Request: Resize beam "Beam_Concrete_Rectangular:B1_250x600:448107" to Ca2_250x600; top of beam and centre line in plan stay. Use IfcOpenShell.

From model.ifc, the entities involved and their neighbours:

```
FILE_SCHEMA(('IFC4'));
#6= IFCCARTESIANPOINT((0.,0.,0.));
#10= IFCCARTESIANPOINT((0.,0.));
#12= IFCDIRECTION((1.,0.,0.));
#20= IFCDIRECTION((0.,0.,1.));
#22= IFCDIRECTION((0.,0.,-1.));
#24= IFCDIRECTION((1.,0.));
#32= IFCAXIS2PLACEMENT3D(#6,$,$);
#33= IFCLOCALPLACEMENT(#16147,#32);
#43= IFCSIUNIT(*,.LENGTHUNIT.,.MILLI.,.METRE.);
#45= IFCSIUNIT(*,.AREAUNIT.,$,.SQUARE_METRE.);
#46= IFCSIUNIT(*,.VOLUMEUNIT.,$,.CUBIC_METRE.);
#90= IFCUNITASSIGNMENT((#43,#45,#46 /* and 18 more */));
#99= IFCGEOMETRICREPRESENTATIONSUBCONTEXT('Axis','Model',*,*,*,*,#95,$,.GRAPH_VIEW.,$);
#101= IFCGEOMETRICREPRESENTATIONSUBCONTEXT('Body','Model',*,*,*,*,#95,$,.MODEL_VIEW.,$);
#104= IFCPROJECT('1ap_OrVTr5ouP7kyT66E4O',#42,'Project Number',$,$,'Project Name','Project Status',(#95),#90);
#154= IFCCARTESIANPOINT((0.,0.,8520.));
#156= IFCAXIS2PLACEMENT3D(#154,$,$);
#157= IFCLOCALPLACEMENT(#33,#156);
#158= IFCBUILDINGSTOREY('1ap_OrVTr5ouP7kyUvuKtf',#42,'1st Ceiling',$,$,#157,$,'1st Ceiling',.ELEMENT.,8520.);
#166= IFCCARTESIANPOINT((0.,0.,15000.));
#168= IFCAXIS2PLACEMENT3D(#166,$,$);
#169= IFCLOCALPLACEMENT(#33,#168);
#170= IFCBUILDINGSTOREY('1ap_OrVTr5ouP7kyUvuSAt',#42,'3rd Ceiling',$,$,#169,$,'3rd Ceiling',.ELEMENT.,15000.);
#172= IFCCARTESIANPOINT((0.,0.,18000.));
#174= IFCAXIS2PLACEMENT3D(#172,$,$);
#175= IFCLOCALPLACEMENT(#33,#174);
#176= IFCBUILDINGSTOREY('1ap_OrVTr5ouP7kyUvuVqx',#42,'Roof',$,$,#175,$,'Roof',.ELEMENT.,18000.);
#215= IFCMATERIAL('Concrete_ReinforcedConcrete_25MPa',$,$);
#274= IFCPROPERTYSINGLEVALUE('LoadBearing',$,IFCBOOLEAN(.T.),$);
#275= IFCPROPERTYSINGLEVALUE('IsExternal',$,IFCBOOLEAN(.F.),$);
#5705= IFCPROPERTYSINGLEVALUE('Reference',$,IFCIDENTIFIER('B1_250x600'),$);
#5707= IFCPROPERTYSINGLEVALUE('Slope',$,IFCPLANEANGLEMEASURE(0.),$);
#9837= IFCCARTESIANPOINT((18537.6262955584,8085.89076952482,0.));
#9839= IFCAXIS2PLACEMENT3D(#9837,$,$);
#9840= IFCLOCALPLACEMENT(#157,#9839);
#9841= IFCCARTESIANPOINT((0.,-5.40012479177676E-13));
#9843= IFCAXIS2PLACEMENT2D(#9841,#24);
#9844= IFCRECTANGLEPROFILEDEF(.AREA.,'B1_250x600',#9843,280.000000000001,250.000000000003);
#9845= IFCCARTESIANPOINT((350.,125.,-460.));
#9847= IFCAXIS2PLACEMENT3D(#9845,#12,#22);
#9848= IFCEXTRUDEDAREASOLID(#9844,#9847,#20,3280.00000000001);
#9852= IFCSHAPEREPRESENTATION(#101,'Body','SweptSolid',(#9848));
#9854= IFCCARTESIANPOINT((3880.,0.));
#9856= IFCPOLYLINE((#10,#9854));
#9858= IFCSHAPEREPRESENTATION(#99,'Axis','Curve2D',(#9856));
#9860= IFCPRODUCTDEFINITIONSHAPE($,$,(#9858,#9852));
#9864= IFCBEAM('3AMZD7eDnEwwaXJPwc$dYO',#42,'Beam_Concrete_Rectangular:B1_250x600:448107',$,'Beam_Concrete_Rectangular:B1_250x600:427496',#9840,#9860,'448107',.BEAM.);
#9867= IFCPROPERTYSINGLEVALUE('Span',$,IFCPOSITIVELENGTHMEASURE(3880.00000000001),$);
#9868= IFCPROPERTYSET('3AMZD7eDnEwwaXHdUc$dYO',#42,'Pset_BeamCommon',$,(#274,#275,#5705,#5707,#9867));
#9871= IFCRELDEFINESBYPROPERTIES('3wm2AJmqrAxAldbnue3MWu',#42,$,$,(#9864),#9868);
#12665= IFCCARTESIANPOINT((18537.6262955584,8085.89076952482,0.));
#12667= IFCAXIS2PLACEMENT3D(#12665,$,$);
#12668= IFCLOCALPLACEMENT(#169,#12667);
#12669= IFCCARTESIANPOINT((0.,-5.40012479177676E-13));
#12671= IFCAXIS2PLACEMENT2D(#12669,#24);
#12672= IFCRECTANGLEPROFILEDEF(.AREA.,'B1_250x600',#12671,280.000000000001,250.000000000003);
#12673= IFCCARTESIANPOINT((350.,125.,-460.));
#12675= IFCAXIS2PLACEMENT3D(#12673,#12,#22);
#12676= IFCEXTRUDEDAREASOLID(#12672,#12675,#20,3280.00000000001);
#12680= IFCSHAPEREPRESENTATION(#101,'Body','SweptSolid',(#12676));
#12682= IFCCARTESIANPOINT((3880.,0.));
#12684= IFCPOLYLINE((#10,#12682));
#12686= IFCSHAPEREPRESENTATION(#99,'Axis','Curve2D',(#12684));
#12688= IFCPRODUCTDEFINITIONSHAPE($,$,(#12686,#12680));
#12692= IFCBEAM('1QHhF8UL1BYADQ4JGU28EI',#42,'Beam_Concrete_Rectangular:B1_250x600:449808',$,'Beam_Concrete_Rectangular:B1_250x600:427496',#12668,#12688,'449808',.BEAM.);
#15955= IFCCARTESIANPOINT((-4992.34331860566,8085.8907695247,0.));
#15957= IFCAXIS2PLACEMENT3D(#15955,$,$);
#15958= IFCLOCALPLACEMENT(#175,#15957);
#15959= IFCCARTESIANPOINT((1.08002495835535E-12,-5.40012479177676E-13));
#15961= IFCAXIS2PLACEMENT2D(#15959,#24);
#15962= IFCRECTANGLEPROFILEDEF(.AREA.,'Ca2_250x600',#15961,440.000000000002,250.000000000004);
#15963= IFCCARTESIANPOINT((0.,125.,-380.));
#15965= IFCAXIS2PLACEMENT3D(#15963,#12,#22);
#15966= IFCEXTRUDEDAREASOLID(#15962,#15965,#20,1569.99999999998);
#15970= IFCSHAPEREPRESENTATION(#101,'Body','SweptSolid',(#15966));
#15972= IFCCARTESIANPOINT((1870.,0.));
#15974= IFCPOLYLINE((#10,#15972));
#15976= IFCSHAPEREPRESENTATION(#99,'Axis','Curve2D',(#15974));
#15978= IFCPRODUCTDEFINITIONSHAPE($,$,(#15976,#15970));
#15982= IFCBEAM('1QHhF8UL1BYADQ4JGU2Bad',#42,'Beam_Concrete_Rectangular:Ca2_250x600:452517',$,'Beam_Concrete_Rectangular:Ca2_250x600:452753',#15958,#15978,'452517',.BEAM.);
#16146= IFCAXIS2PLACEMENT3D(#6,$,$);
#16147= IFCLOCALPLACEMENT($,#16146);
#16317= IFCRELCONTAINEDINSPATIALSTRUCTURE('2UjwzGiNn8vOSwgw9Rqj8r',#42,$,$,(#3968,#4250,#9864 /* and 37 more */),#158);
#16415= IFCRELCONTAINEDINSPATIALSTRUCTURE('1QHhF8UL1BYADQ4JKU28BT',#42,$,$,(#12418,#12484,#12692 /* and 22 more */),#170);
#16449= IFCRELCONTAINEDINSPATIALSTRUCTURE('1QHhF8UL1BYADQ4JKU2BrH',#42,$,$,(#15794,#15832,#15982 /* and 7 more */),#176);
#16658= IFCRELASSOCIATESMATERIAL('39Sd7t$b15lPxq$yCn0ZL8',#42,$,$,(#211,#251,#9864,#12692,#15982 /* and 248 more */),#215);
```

```python
import ifcopenshell
import ifcopenshell.api.pset
import ifcopenshell.util.element
import ifcopenshell.util.representation

model = ifcopenshell.open("model.ifc")

member = model.by_id(9864)
source = next(p for p in model.by_type("IfcRectangleProfileDef") if p.ProfileName == "Ca2_250x600")

body = ifcopenshell.util.representation.get_representation(member, "Model", "Body")
solid = body.Items[0]
old_profile = solid.SweptArea

# Copy the section's sizes but keep this member's own profile position.
profile = ifcopenshell.util.element.copy(model, source)
# Profiles are centred, so shift by half the change in depth to hold the top.
shift = (old_profile.XDim - profile.XDim) / 2
x, y = old_profile.Position.Location.Coordinates
up = (-1.0, 0.0)  # upwards, in the solid's own plane
location = model.createIfcCartesianPoint((x + up[0] * shift, y + up[1] * shift))
profile.Position = model.createIfcAxis2Placement2D(location, old_profile.Position.RefDirection)
solid.SweptArea = profile
if not model.get_total_inverses(old_profile):
    ifcopenshell.util.element.remove_deep2(model, old_profile)
member.Name = member.Name.replace("B1_250x600", "Ca2_250x600")
member.ObjectType = member.ObjectType.replace("B1_250x600", "Ca2_250x600")
pset = model.by_id(ifcopenshell.util.element.get_pset(member, "Pset_BeamCommon", should_inherit=False)["id"])
ifcopenshell.api.pset.edit_pset(model, pset=pset, properties={"Reference": "Ca2_250x600"})

print(solid.SweptArea)

model.write("model_v2.ifc")
```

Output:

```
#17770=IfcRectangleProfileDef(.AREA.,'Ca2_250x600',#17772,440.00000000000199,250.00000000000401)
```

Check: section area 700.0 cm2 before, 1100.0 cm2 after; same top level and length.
